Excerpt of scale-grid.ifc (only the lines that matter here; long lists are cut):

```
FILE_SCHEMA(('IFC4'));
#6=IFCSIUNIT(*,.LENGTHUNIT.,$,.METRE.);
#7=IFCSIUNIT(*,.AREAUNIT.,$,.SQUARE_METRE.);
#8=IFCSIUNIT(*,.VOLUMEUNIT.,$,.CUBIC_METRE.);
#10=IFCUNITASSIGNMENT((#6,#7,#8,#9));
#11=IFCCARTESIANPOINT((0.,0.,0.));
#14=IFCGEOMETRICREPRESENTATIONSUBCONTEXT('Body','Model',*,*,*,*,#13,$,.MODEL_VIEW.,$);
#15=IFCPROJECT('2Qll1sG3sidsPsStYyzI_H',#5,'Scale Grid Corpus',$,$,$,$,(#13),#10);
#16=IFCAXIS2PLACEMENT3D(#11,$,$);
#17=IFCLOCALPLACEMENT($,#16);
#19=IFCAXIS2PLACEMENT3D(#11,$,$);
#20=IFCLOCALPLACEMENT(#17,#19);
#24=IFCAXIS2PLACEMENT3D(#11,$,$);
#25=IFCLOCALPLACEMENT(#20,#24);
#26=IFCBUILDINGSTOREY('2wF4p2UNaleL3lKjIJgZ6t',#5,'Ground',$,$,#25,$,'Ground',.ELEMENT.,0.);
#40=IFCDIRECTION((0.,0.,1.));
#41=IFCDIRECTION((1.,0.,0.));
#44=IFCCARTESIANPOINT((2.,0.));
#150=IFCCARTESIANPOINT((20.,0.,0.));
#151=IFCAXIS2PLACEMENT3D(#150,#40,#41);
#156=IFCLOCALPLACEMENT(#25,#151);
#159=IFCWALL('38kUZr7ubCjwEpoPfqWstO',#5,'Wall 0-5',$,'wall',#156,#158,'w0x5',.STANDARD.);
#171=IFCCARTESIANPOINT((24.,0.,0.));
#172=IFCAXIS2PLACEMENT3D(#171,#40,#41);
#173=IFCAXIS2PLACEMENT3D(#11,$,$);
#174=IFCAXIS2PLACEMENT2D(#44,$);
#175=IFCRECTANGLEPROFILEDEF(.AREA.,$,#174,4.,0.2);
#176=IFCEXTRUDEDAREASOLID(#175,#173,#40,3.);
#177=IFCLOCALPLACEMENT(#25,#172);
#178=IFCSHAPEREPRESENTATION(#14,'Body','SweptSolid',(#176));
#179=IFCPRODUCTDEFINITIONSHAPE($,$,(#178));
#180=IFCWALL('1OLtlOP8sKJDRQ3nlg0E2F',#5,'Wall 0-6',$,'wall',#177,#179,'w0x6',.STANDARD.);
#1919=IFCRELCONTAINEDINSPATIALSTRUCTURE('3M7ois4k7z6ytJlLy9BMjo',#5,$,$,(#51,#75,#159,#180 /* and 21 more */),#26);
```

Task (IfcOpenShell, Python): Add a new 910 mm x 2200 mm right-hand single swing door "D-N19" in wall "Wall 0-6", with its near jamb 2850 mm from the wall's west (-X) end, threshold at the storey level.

```python
import numpy as np
import ifcopenshell
import ifcopenshell.api.feature
import ifcopenshell.api.geometry
import ifcopenshell.api.root
import ifcopenshell.api.spatial
import ifcopenshell.geom
import ifcopenshell.util.element
import ifcopenshell.util.placement
import ifcopenshell.util.representation
import ifcopenshell.util.shape
import ifcopenshell.util.unit

model = ifcopenshell.open("scale-grid.ifc")
unit_scale = ifcopenshell.util.unit.calculate_unit_scale(model)
settings = ifcopenshell.geom.settings()


def volume(element):
    """Net volume in cubic metres, openings subtracted."""
    shape = ifcopenshell.geom.create_shape(settings, element)
    return ifcopenshell.util.shape.get_volume(shape.geometry)


wall = model.by_id(180)
storey = ifcopenshell.util.element.get_container(wall, ifc_class="IfcBuildingStorey")
context = ifcopenshell.util.representation.get_context(model, "Model", "Body", "MODEL_VIEW")
before = volume(wall)

width, height, from_end, sill = 0.91, 2.2, 2.85, 0.0  # metres

# The wall runs along its own X axis, and the end named is its -X end.
wall_shape = ifcopenshell.geom.create_shape(settings, wall)
x, y, z = ifcopenshell.util.shape.get_vertices(wall_shape.geometry).T
start = x.min() + from_end
face, thickness = float(y.min()), float(y.max() - y.min())
wall_matrix = ifcopenshell.util.placement.get_local_placement(wall.ObjectPlacement)
level = ifcopenshell.util.placement.get_local_placement(storey.ObjectPlacement)[2, 3]


def in_wall(x, y):
    """Placement at x, y metres in the wall's axes, at sill height."""
    matrix = wall_matrix.copy()
    matrix[:, 3] = wall_matrix @ np.array([x / unit_scale, y / unit_scale, 0.0, 1.0])
    matrix[2, 3] = level + sill / unit_scale
    return matrix


# Opening: a box that overshoots both wall faces by 50 mm.
opening = ifcopenshell.api.root.create_entity(model, ifc_class="IfcOpeningElement", predefined_type="OPENING")
box = ifcopenshell.api.geometry.add_wall_representation(
    model, context=context, length=width, height=height, thickness=thickness + 0.1
)
ifcopenshell.api.geometry.assign_representation(model, product=opening, representation=box)
ifcopenshell.api.geometry.edit_object_placement(model, product=opening, matrix=in_wall(start, face - 0.05), is_si=False)
ifcopenshell.api.feature.add_feature(model, feature=opening, element=wall)

door = ifcopenshell.api.root.create_entity(model, ifc_class="IfcDoor", name="D-N19", predefined_type="DOOR")
door.OverallWidth, door.OverallHeight = width / unit_scale, height / unit_scale
door.OperationType = "SINGLE_SWING_RIGHT"
body = ifcopenshell.api.geometry.add_door_representation(
    model,
    context=context,
    overall_width=door.OverallWidth,
    overall_height=door.OverallHeight,
    operation_type="SINGLE_SWING_RIGHT",
    lining_properties={"LiningDepth": thickness / unit_scale, "ThresholdDepth": thickness / unit_scale},
)
ifcopenshell.api.geometry.assign_representation(model, product=door, representation=body)
ifcopenshell.api.spatial.assign_container(model, products=[door], relating_structure=storey)
ifcopenshell.api.feature.add_filling(model, opening=opening, element=door)

# The lining spans the wall, so the door starts at the wall face.
ifcopenshell.api.geometry.edit_object_placement(model, product=door, matrix=in_wall(start, face), is_si=False)

after = volume(wall)

print(f"wall volume {before:.3f} -> {after:.3f} m3")

model.write("scale-grid_edited.ifc")
```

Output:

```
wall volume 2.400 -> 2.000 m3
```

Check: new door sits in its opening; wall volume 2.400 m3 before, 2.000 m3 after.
